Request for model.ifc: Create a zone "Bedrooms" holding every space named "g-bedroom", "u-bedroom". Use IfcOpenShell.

First a look at what the model holds.

```python
import ifcopenshell

model = ifcopenshell.open("model.ifc")
print(model.schema)
seen = {}
for space in model.by_type("IfcSpace"):
    seen[space.LongName] = seen.get(space.LongName, 0) + 1
for name, count in sorted(seen.items(), key=str):
    print(count, "x", name)
print("zones:", [z.Name for z in model.by_type("IfcZone")][:20])
```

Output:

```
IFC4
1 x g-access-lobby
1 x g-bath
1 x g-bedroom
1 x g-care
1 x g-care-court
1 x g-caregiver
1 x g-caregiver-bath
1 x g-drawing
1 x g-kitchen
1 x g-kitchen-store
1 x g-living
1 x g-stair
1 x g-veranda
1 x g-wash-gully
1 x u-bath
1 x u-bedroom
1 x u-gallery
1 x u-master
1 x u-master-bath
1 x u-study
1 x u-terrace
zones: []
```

```python
import ifcopenshell
import ifcopenshell.api.group
import ifcopenshell.api.root

model = ifcopenshell.open("model.ifc")

names = {"g-bedroom", "u-bedroom"}
spaces = [s for s in model.by_type("IfcSpace") if s.LongName in names]

zone = ifcopenshell.api.root.create_entity(model, ifc_class="IfcZone", name="Bedrooms")
ifcopenshell.api.group.assign_group(model, products=spaces, group=zone)
print(len(spaces), "spaces in", zone.Name)

model.write("model_v2.ifc")
```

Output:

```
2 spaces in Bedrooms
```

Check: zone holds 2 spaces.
